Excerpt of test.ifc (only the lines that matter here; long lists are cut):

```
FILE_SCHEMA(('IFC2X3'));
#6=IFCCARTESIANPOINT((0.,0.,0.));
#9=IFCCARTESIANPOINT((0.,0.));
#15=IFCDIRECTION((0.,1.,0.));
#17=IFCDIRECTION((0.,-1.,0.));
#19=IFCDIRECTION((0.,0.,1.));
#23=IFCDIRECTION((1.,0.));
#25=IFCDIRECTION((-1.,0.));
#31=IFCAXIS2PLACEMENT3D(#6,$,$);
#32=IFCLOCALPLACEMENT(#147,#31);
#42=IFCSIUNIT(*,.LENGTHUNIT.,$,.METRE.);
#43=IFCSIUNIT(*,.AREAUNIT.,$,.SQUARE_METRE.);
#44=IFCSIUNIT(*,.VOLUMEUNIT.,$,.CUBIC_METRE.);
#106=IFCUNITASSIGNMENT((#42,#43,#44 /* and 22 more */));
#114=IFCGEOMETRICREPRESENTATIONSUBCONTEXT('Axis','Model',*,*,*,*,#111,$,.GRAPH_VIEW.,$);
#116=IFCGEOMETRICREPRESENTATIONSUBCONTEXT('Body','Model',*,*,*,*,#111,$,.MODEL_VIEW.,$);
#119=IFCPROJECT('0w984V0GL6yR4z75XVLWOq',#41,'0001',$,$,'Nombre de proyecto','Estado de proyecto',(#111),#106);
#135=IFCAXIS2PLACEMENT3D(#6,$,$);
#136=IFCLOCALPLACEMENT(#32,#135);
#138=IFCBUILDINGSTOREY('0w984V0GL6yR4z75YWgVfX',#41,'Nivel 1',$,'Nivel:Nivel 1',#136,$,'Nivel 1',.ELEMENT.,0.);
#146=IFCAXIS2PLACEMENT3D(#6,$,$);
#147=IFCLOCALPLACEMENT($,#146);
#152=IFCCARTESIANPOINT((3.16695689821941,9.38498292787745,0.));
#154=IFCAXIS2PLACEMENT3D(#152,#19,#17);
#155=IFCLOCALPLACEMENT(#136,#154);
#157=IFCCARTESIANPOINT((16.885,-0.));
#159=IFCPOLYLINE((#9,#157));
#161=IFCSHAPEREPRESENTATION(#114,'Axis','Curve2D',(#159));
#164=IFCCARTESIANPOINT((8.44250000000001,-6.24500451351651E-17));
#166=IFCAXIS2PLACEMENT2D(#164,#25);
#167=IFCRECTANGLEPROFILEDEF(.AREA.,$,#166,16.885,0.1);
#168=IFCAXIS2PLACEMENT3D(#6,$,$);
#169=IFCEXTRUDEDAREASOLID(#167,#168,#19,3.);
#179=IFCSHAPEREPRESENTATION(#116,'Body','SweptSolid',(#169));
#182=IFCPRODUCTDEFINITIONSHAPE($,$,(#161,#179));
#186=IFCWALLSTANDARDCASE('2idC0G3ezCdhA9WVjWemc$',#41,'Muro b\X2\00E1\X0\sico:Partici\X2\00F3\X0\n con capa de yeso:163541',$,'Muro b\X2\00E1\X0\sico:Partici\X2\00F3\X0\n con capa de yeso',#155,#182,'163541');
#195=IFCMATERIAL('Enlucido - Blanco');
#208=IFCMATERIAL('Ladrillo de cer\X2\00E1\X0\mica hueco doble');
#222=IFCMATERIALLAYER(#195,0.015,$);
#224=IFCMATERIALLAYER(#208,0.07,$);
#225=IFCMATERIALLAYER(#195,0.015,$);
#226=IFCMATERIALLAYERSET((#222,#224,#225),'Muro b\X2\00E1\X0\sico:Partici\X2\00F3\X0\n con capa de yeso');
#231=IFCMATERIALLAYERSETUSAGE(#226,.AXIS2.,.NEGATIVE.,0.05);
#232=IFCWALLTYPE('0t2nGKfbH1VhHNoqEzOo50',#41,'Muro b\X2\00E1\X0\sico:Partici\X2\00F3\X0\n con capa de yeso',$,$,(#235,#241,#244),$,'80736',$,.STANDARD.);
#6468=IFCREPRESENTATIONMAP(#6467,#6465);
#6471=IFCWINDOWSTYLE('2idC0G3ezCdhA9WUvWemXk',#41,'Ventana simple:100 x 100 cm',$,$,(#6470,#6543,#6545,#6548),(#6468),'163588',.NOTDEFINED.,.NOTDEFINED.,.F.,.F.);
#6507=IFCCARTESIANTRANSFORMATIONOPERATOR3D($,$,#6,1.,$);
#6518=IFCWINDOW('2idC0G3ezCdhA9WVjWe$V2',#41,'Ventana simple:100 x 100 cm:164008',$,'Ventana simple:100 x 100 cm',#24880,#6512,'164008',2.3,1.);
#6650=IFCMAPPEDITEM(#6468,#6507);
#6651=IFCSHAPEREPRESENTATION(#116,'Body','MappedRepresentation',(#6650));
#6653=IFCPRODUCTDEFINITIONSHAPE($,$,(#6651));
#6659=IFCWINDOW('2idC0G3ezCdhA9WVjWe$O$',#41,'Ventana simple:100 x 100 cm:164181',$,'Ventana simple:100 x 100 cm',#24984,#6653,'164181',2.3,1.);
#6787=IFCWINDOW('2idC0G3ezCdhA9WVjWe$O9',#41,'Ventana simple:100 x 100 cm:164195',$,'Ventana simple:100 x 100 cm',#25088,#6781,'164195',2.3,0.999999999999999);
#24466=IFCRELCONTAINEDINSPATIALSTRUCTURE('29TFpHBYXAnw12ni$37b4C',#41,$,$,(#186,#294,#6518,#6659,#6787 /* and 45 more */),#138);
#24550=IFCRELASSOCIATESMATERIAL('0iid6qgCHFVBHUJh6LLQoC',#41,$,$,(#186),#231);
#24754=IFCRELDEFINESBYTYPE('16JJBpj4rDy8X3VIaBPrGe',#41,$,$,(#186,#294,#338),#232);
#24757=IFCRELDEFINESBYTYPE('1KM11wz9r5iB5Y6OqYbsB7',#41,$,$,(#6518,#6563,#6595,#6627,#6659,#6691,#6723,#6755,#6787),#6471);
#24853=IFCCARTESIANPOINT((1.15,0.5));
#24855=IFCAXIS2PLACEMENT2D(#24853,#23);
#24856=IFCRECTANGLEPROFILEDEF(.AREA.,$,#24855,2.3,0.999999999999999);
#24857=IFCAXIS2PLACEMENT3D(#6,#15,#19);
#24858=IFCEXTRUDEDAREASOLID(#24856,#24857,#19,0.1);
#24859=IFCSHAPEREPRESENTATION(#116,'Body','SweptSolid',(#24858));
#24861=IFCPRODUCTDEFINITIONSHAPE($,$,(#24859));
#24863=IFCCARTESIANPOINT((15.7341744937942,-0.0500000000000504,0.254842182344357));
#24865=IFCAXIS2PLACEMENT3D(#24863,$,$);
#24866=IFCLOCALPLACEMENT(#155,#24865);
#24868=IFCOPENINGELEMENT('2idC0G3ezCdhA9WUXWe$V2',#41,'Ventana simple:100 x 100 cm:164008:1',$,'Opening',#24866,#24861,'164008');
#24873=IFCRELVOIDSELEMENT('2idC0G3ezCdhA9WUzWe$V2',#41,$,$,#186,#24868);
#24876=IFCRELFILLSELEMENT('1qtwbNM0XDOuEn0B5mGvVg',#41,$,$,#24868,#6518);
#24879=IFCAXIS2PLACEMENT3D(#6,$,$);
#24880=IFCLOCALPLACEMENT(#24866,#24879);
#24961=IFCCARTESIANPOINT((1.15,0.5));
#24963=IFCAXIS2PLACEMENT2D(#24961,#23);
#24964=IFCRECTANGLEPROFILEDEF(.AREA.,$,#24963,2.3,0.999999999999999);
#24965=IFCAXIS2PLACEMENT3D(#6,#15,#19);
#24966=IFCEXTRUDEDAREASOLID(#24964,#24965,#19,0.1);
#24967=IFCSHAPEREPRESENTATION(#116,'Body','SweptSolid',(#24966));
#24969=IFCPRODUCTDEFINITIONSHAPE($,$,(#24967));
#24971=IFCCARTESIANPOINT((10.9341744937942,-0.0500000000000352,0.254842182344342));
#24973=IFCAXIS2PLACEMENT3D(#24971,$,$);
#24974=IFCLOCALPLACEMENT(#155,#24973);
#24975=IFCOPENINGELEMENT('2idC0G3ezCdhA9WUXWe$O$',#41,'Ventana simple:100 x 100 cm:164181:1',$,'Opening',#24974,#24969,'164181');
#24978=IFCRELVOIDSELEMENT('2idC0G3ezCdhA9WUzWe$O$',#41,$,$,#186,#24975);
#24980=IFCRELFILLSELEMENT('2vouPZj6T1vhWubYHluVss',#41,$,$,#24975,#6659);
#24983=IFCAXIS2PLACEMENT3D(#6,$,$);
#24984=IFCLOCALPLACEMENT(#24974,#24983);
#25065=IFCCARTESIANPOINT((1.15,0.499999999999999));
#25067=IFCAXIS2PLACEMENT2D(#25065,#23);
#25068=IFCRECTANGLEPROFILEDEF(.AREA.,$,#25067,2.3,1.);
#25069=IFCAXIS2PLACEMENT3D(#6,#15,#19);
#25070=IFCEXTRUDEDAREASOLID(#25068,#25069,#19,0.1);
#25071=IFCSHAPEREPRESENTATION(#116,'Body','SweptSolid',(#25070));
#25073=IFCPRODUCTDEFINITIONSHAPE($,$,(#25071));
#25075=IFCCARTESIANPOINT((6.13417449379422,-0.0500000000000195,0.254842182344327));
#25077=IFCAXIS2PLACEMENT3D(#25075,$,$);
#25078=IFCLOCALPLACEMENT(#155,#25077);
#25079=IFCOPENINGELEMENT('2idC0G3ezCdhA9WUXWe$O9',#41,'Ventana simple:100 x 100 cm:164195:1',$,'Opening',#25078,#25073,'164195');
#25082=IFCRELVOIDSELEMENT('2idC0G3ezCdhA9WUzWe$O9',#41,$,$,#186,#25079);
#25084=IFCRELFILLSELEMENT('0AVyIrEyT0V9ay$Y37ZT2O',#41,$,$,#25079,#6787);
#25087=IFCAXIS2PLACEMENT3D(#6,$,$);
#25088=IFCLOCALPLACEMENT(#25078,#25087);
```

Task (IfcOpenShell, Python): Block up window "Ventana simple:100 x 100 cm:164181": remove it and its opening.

```python
import ifcopenshell
import ifcopenshell.api.feature
import ifcopenshell.api.root
import ifcopenshell.geom
import ifcopenshell.util.shape

model = ifcopenshell.open("test.ifc")
settings = ifcopenshell.geom.settings()


def volume(element):
    """Net volume in cubic metres, openings subtracted."""
    shape = ifcopenshell.geom.create_shape(settings, element)
    return ifcopenshell.util.shape.get_volume(shape.geometry)


window = model.by_guid("2idC0G3ezCdhA9WVjWe$O$")
opening = window.FillsVoids[0].RelatingOpeningElement
wall = opening.VoidsElements[0].RelatingBuildingElement
before = volume(wall)

ifcopenshell.api.root.remove_product(model, product=window)
ifcopenshell.api.feature.remove_feature(model, feature=opening)

after = volume(wall)

print(f"wall volume {before:.3f} -> {after:.3f} m3")

model.write("test_v2.ifc")
```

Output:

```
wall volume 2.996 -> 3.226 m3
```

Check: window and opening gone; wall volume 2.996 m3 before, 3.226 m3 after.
